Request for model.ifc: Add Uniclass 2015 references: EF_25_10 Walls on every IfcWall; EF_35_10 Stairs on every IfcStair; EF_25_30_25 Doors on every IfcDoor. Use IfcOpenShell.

First a look at what the model holds.

```python
import ifcopenshell

model = ifcopenshell.open("model.ifc")
print(model.schema)
print("classifications:", [c.Name for c in model.by_type("IfcClassification")])
for ifc_class in ("IfcDoor", "IfcRoof", "IfcStair", "IfcWall", "IfcWindow"):
    print(ifc_class, len(model.by_type(ifc_class)))
```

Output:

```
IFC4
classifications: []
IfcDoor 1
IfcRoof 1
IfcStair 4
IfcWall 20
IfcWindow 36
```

```python
import ifcopenshell
import ifcopenshell.api.classification

model = ifcopenshell.open("model.ifc")

system = ifcopenshell.api.classification.add_classification(model, classification="Uniclass 2015")

codes = {
    "IfcWall": ("EF_25_10", "Walls"),
    "IfcStair": ("EF_35_10", "Stairs"),
    "IfcDoor": ("EF_25_30_25", "Doors"),
}
for ifc_class, (code, name) in codes.items():
    products = model.by_type(ifc_class)
    ifcopenshell.api.classification.add_reference(
        model, products=products, classification=system, identification=code, name=name
    )
    print(code, len(products))

model.write("model_edited.ifc")
```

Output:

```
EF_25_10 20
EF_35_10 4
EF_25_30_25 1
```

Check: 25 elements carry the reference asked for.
